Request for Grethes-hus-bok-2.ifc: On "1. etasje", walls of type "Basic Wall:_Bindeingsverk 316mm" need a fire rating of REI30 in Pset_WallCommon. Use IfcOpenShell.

First a look at what the model holds.

```python
import ifcopenshell
import ifcopenshell.util.element

model = ifcopenshell.open("Grethes-hus-bok-2.ifc")
print(model.schema)
storey = next(s for s in model.by_type("IfcBuildingStorey") if s.Name == "1. etasje")
walls = [e for e in ifcopenshell.util.element.get_decomposition(storey) if e.is_a("IfcWall")]
seen = {}
for e in walls:
    element_type = ifcopenshell.util.element.get_type(e)
    key = (element_type.Name if element_type != e and element_type else None, ifcopenshell.util.element.get_pset(e, "Pset_WallCommon", "FireRating"))
    seen[key] = seen.get(key, 0) + 1
for (name, value), count in sorted(seen.items(), key=str):
    print(count, "x", name, "|", value)
```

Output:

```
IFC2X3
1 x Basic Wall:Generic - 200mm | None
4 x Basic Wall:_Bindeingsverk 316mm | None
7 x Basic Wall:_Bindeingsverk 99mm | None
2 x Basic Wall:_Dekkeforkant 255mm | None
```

```python
import ifcopenshell
import ifcopenshell.api.pset
import ifcopenshell.util.element

model = ifcopenshell.open("Grethes-hus-bok-2.ifc")

storey = next(s for s in model.by_type("IfcBuildingStorey") if s.Name == "1. etasje")
walls = [e for e in ifcopenshell.util.element.get_decomposition(storey) if e.is_a("IfcWall")]

count = 0
for e in walls:
    element_type = ifcopenshell.util.element.get_type(e)
    if element_type in (None, e) or element_type.Name != "Basic Wall:_Bindeingsverk 316mm":
        continue
    # add_pset returns the element's existing set when there is one.
    pset = ifcopenshell.api.pset.add_pset(model, product=e, name="Pset_WallCommon")
    ifcopenshell.api.pset.edit_pset(model, pset=pset, properties={"FireRating": "REI30"})
    count += 1

print(count, "walls updated")

model.write("Grethes-hus-bok-2_edited.ifc")
```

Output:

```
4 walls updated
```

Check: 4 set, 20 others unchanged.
